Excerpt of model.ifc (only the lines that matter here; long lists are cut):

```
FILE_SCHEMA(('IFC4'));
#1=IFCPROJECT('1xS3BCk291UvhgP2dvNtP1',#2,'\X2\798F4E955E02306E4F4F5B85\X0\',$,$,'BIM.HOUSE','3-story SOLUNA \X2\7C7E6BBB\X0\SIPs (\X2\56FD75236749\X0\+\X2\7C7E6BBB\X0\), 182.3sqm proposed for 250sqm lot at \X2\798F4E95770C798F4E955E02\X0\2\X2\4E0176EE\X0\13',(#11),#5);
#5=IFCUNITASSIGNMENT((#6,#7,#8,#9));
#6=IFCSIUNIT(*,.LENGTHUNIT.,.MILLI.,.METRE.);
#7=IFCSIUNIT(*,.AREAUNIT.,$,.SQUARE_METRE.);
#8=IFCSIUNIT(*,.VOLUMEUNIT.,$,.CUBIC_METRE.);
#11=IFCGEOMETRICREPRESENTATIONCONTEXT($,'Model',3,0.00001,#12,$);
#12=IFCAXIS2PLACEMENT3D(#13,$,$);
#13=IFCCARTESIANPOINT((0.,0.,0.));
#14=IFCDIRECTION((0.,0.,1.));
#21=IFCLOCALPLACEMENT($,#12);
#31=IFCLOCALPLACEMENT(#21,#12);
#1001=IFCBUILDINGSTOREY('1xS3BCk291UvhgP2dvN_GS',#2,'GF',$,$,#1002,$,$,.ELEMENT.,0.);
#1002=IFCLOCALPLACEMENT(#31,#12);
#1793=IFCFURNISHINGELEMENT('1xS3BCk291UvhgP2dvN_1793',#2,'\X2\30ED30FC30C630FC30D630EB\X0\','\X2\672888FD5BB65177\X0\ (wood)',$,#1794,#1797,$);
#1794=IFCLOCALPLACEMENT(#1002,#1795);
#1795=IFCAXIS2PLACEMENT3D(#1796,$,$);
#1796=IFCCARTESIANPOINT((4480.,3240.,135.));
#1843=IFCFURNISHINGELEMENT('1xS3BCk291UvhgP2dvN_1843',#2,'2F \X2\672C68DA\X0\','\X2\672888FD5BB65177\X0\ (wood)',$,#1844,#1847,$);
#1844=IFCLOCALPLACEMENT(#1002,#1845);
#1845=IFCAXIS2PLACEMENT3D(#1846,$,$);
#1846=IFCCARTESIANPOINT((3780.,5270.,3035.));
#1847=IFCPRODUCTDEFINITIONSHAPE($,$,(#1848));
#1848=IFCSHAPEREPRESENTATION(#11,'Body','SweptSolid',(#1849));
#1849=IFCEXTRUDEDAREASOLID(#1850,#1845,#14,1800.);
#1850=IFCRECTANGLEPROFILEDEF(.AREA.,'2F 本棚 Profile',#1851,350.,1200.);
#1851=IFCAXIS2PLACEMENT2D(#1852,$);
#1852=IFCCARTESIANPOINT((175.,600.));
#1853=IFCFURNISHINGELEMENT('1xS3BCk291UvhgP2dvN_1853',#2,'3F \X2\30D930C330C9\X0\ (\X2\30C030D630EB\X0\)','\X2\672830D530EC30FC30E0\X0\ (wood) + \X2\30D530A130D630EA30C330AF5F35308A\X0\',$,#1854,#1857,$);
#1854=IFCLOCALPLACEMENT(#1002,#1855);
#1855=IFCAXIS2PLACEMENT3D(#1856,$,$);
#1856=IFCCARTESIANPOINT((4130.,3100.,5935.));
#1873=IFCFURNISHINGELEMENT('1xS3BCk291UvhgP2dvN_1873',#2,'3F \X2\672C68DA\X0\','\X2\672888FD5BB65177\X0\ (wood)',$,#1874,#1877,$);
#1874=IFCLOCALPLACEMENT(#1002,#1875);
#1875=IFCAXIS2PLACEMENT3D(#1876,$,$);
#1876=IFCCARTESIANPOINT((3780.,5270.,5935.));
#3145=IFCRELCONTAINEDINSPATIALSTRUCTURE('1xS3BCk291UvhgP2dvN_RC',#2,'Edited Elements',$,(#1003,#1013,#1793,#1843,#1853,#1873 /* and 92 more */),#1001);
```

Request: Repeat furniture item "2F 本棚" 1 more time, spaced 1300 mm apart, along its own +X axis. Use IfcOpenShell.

```python
import ifcopenshell
import ifcopenshell.api.geometry
import ifcopenshell.api.root
import ifcopenshell.util.element
import ifcopenshell.util.placement
import ifcopenshell.util.unit

model = ifcopenshell.open("model.ifc")
unit_scale = ifcopenshell.util.unit.calculate_unit_scale(model)


def reuse_history(source, copy):
    """copy_class also copies each property set's owner history, people and application; keep the originals."""
    for rel in copy.IsDefinedBy:
        if rel.is_a("IfcRelDefinesByProperties") and (history := rel.RelatingPropertyDefinition.OwnerHistory):
            rel.RelatingPropertyDefinition.OwnerHistory = source.OwnerHistory
            ifcopenshell.util.element.remove_deep2(model, history)


source = model.by_guid("1xS3BCk291UvhgP2dvN_1843")
base = ifcopenshell.util.placement.get_local_placement(source.ObjectPlacement)
step = base[:3, 0] * 1.3 / unit_scale

for i in range(1, 2):
    copy = ifcopenshell.api.root.copy_class(model, product=source)
    copy.Representation = ifcopenshell.util.element.copy_deep(
        model, source.Representation, exclude=["IfcGeometricRepresentationContext", "IfcRepresentationMap"]
    )
    reuse_history(source, copy)
    matrix = base.copy()
    matrix[:3, 3] += i * step
    print("added at", matrix[:3, 3].round(3) + 0.0)
    ifcopenshell.api.geometry.edit_object_placement(model, product=copy, matrix=matrix, is_si=False)

model.write("model_updated.ifc")
```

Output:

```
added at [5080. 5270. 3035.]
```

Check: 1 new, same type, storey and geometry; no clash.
